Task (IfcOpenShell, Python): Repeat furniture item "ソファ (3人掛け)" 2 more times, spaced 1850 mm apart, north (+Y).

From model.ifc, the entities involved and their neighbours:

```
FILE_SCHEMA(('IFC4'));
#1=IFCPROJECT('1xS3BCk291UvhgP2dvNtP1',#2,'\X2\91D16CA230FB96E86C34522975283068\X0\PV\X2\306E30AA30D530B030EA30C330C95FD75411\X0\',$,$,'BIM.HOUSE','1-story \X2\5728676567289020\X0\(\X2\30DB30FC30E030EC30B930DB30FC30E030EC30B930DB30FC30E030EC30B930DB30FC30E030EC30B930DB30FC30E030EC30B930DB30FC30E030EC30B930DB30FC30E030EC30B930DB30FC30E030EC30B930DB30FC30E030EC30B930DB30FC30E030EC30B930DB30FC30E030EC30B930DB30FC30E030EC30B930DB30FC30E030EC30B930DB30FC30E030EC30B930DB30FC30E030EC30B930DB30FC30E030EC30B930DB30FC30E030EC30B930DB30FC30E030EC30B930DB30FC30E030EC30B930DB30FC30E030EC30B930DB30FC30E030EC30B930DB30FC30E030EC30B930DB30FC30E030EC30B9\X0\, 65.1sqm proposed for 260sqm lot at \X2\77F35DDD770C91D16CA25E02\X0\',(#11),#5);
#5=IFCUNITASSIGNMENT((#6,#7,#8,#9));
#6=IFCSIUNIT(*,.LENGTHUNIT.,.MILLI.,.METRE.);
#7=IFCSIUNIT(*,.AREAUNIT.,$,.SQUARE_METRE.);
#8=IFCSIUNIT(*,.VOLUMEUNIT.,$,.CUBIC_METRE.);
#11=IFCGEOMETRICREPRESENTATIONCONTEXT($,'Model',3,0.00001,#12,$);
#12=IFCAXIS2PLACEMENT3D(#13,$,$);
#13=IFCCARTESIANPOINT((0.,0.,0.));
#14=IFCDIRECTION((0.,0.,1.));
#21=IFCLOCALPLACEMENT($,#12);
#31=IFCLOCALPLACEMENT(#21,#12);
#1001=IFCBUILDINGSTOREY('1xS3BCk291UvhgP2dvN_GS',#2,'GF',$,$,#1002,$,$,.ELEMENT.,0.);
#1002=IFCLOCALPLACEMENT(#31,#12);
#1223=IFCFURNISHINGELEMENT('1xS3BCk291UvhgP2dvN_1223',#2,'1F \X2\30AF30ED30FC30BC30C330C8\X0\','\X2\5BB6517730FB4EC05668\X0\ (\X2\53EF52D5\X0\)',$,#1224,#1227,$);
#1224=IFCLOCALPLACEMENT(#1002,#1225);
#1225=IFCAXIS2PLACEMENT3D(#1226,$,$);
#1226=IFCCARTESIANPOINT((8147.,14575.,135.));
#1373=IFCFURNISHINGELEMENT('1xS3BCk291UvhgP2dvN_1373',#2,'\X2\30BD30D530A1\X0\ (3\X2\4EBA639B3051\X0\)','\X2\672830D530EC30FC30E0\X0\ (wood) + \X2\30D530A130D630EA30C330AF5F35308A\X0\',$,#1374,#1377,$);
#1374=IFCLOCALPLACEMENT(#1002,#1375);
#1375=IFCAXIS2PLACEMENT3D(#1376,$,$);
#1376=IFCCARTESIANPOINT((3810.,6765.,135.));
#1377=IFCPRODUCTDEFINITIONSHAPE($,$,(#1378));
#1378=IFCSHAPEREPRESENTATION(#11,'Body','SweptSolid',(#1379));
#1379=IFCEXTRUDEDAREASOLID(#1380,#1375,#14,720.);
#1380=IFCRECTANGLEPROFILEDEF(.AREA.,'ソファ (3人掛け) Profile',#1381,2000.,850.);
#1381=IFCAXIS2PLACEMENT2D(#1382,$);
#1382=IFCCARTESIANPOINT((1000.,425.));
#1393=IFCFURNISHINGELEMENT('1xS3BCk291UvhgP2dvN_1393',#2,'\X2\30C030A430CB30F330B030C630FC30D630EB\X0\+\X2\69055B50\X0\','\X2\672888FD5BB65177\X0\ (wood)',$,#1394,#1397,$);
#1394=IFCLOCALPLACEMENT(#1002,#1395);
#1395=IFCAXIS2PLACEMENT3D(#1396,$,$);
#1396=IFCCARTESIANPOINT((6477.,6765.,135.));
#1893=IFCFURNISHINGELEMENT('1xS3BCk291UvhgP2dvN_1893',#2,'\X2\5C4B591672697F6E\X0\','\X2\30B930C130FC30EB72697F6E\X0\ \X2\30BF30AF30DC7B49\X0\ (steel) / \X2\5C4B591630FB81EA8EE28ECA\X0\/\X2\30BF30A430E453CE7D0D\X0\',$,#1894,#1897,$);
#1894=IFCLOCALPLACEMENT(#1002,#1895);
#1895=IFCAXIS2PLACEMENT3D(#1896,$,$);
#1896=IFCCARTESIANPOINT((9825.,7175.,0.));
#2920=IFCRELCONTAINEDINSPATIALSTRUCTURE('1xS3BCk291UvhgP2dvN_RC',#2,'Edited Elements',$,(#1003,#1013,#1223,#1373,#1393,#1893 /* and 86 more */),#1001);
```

```python
import numpy as np
import ifcopenshell
import ifcopenshell.api.geometry
import ifcopenshell.api.root
import ifcopenshell.util.element
import ifcopenshell.util.placement

model = ifcopenshell.open("model.ifc")


def reuse_history(source, copy):
    """copy_class also copies each property set's owner history, people and application; keep the originals."""
    for rel in copy.IsDefinedBy:
        if rel.is_a("IfcRelDefinesByProperties") and (history := rel.RelatingPropertyDefinition.OwnerHistory):
            rel.RelatingPropertyDefinition.OwnerHistory = source.OwnerHistory
            ifcopenshell.util.element.remove_deep2(model, history)


source = model.by_id(1373)
base = ifcopenshell.util.placement.get_local_placement(source.ObjectPlacement)
step = np.array([0.0, 1.0, 0.0]) * 1850.0

for i in range(1, 3):
    copy = ifcopenshell.api.root.copy_class(model, product=source)
    copy.Representation = ifcopenshell.util.element.copy_deep(
        model, source.Representation, exclude=["IfcGeometricRepresentationContext", "IfcRepresentationMap"]
    )
    reuse_history(source, copy)
    matrix = base.copy()
    matrix[:3, 3] += i * step
    print("added at", matrix[:3, 3].round(3) + 0.0)
    ifcopenshell.api.geometry.edit_object_placement(model, product=copy, matrix=matrix, is_si=False)

model.write("model-out.ifc")
```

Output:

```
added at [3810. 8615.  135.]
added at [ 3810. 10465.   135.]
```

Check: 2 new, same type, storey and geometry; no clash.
